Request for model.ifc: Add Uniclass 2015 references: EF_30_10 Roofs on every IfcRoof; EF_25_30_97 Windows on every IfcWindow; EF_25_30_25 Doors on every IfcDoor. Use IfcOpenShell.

First a look at what the model holds.

```python
import ifcopenshell

model = ifcopenshell.open("model.ifc")
print(model.schema)
print("classifications:", [c.Name for c in model.by_type("IfcClassification")])
for ifc_class in ("IfcDoor", "IfcRoof", "IfcStair", "IfcWall", "IfcWindow"):
    print(ifc_class, len(model.by_type(ifc_class)))
```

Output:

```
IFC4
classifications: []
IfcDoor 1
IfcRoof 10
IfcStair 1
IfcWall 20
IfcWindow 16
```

```python
import ifcopenshell
import ifcopenshell.api.classification

model = ifcopenshell.open("model.ifc")

system = ifcopenshell.api.classification.add_classification(model, classification="Uniclass 2015")

codes = {
    "IfcRoof": ("EF_30_10", "Roofs"),
    "IfcWindow": ("EF_25_30_97", "Windows"),
    "IfcDoor": ("EF_25_30_25", "Doors"),
}
for ifc_class, (code, name) in codes.items():
    products = model.by_type(ifc_class)
    ifcopenshell.api.classification.add_reference(
        model, products=products, classification=system, identification=code, name=name
    )
    print(code, len(products))

model.write("model_rev.ifc")
```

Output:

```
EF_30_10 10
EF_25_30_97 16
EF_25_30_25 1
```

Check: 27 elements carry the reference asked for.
